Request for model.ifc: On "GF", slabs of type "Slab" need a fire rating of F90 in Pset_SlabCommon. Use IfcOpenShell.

First a look at what the model holds.

```python
import ifcopenshell
import ifcopenshell.util.element

model = ifcopenshell.open("model.ifc")
print(model.schema)
storey = next(s for s in model.by_type("IfcBuildingStorey") if s.Name == "GF")
slabs = [e for e in ifcopenshell.util.element.get_decomposition(storey) if e.is_a("IfcSlab")]
seen = {}
for e in slabs:
    element_type = ifcopenshell.util.element.get_type(e)
    key = (element_type.Name if element_type != e and element_type else None, ifcopenshell.util.element.get_pset(e, "Pset_SlabCommon", "FireRating"))
    seen[key] = seen.get(key, 0) + 1
for (name, value), count in sorted(seen.items(), key=str):
    print(count, "x", name, "|", value)
```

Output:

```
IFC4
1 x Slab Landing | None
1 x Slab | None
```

```python
import ifcopenshell
import ifcopenshell.api.pset
import ifcopenshell.util.element

model = ifcopenshell.open("model.ifc")

storey = next(s for s in model.by_type("IfcBuildingStorey") if s.Name == "GF")
slabs = [e for e in ifcopenshell.util.element.get_decomposition(storey) if e.is_a("IfcSlab")]

count = 0
for e in slabs:
    element_type = ifcopenshell.util.element.get_type(e)
    if element_type in (None, e) or element_type.Name != "Slab":
        continue
    # add_pset returns the element's existing set when there is one.
    pset = ifcopenshell.api.pset.add_pset(model, product=e, name="Pset_SlabCommon")
    ifcopenshell.api.pset.edit_pset(model, pset=pset, properties={"FireRating": "F90"})
    count += 1

print(count, "slabs updated")

model.write("model_rev.ifc")
```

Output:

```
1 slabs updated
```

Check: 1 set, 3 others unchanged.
